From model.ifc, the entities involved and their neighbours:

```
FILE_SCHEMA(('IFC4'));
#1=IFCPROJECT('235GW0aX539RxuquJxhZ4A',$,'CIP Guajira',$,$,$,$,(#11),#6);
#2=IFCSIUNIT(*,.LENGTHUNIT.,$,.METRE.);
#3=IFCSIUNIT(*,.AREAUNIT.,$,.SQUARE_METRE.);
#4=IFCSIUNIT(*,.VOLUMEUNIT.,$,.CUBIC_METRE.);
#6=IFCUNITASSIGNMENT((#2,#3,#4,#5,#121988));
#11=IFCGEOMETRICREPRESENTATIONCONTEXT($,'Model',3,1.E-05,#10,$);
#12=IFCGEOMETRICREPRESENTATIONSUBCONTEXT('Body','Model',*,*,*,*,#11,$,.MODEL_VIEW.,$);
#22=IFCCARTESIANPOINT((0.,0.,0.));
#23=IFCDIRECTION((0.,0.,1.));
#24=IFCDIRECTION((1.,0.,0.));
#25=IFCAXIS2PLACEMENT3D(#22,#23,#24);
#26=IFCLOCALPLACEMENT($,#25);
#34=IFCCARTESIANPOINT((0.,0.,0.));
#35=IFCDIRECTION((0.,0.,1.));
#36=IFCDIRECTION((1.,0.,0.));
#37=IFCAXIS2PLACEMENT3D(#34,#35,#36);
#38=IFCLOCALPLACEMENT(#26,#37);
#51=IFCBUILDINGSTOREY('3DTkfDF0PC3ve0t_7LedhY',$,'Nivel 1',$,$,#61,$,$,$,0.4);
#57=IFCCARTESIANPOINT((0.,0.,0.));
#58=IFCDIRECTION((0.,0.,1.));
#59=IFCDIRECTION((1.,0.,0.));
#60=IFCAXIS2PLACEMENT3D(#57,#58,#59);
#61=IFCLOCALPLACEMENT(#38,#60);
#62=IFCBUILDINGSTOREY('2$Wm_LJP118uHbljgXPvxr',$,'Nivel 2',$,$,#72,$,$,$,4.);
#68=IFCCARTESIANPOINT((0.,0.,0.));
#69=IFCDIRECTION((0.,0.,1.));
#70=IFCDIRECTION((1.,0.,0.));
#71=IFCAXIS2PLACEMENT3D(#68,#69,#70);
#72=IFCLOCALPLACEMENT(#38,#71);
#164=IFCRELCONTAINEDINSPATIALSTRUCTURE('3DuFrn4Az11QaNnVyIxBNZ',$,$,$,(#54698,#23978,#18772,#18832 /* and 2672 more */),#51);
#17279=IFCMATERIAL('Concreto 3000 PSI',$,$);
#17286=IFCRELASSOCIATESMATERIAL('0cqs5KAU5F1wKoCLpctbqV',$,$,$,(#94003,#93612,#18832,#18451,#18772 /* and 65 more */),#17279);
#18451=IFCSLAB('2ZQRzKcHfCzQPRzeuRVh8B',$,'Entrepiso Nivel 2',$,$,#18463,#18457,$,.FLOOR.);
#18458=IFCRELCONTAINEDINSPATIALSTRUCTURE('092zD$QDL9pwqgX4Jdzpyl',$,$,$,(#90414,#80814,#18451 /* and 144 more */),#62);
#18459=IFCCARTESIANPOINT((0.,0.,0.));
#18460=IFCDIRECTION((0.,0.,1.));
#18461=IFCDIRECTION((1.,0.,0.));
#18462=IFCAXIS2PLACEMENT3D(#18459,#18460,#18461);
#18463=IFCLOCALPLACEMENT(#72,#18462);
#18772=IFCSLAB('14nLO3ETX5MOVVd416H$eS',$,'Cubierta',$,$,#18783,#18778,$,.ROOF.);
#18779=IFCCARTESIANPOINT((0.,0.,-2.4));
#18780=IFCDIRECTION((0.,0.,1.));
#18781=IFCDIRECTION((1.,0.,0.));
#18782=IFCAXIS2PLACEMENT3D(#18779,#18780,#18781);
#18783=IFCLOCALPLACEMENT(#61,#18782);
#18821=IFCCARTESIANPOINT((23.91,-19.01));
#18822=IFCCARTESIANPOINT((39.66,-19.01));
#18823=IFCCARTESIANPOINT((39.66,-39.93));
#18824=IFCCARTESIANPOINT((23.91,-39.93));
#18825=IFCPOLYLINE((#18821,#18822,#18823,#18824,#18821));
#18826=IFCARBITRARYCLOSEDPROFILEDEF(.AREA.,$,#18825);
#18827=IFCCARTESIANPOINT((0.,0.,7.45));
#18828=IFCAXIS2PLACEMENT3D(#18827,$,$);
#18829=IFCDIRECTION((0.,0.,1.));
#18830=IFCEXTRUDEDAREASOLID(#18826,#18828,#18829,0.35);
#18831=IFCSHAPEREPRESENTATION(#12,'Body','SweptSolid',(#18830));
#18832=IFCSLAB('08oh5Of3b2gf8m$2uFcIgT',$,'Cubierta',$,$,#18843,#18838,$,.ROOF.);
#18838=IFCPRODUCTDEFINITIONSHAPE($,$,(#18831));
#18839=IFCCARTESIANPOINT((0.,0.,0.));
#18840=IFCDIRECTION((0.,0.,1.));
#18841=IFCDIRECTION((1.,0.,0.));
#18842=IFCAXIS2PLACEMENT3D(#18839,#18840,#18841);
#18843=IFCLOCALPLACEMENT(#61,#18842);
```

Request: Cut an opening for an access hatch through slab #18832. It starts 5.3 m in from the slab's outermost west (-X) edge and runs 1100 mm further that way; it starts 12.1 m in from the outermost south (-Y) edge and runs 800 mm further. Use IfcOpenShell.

```python
import numpy as np
import ifcopenshell
import ifcopenshell.api.feature
import ifcopenshell.api.geometry
import ifcopenshell.api.root
import ifcopenshell.geom
import ifcopenshell.util.placement
import ifcopenshell.util.representation
import ifcopenshell.util.shape
import ifcopenshell.util.unit

model = ifcopenshell.open("model.ifc")
unit_scale = ifcopenshell.util.unit.calculate_unit_scale(model)
settings = ifcopenshell.geom.settings()


def volume(element):
    """Net volume in cubic metres, openings subtracted."""
    shape = ifcopenshell.geom.create_shape(settings, element)
    return ifcopenshell.util.shape.get_volume(shape.geometry)


slab = model.by_id(18832)
before = volume(slab)

# Extent in the slab's own axes, in metres. The edges named are its -X and -Y sides.
slab_shape = ifcopenshell.geom.create_shape(settings, slab)
vertices = ifcopenshell.util.shape.get_vertices(slab_shape.geometry)
x_min, y_min, bottom = vertices.min(axis=0)
top = vertices[:, 2].max()

opening = ifcopenshell.api.root.create_entity(model, ifc_class="IfcOpeningElement", name="Access hatch opening", predefined_type="OPENING")
context = ifcopenshell.util.representation.get_context(model, "Model", "Body", "MODEL_VIEW")
width, depth = 1.1, 0.8
outline = [(0.0, 0.0), (width, 0.0), (width, depth), (0.0, depth), (0.0, 0.0)]
# Overshoot both faces by 50 mm so the cut is clean.
shape = ifcopenshell.api.geometry.add_slab_representation(
    model, context=context, depth=top - bottom + 0.1, polyline=outline
)
ifcopenshell.api.geometry.assign_representation(model, product=opening, representation=shape)

matrix = ifcopenshell.util.placement.get_local_placement(slab.ObjectPlacement)
matrix[:, 3] = matrix @ np.append(np.array([x_min + 5.3, y_min + 12.1, bottom - 0.05]) / unit_scale, 1.0)
ifcopenshell.api.geometry.edit_object_placement(model, product=opening, matrix=matrix, is_si=False)
ifcopenshell.api.feature.add_feature(model, feature=opening, element=slab)

after = volume(slab)

print(f"slab volume {before:.3f} -> {after:.3f} m3")

model.write("model_rev.ifc")
```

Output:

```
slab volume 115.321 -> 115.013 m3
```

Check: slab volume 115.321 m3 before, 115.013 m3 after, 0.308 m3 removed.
